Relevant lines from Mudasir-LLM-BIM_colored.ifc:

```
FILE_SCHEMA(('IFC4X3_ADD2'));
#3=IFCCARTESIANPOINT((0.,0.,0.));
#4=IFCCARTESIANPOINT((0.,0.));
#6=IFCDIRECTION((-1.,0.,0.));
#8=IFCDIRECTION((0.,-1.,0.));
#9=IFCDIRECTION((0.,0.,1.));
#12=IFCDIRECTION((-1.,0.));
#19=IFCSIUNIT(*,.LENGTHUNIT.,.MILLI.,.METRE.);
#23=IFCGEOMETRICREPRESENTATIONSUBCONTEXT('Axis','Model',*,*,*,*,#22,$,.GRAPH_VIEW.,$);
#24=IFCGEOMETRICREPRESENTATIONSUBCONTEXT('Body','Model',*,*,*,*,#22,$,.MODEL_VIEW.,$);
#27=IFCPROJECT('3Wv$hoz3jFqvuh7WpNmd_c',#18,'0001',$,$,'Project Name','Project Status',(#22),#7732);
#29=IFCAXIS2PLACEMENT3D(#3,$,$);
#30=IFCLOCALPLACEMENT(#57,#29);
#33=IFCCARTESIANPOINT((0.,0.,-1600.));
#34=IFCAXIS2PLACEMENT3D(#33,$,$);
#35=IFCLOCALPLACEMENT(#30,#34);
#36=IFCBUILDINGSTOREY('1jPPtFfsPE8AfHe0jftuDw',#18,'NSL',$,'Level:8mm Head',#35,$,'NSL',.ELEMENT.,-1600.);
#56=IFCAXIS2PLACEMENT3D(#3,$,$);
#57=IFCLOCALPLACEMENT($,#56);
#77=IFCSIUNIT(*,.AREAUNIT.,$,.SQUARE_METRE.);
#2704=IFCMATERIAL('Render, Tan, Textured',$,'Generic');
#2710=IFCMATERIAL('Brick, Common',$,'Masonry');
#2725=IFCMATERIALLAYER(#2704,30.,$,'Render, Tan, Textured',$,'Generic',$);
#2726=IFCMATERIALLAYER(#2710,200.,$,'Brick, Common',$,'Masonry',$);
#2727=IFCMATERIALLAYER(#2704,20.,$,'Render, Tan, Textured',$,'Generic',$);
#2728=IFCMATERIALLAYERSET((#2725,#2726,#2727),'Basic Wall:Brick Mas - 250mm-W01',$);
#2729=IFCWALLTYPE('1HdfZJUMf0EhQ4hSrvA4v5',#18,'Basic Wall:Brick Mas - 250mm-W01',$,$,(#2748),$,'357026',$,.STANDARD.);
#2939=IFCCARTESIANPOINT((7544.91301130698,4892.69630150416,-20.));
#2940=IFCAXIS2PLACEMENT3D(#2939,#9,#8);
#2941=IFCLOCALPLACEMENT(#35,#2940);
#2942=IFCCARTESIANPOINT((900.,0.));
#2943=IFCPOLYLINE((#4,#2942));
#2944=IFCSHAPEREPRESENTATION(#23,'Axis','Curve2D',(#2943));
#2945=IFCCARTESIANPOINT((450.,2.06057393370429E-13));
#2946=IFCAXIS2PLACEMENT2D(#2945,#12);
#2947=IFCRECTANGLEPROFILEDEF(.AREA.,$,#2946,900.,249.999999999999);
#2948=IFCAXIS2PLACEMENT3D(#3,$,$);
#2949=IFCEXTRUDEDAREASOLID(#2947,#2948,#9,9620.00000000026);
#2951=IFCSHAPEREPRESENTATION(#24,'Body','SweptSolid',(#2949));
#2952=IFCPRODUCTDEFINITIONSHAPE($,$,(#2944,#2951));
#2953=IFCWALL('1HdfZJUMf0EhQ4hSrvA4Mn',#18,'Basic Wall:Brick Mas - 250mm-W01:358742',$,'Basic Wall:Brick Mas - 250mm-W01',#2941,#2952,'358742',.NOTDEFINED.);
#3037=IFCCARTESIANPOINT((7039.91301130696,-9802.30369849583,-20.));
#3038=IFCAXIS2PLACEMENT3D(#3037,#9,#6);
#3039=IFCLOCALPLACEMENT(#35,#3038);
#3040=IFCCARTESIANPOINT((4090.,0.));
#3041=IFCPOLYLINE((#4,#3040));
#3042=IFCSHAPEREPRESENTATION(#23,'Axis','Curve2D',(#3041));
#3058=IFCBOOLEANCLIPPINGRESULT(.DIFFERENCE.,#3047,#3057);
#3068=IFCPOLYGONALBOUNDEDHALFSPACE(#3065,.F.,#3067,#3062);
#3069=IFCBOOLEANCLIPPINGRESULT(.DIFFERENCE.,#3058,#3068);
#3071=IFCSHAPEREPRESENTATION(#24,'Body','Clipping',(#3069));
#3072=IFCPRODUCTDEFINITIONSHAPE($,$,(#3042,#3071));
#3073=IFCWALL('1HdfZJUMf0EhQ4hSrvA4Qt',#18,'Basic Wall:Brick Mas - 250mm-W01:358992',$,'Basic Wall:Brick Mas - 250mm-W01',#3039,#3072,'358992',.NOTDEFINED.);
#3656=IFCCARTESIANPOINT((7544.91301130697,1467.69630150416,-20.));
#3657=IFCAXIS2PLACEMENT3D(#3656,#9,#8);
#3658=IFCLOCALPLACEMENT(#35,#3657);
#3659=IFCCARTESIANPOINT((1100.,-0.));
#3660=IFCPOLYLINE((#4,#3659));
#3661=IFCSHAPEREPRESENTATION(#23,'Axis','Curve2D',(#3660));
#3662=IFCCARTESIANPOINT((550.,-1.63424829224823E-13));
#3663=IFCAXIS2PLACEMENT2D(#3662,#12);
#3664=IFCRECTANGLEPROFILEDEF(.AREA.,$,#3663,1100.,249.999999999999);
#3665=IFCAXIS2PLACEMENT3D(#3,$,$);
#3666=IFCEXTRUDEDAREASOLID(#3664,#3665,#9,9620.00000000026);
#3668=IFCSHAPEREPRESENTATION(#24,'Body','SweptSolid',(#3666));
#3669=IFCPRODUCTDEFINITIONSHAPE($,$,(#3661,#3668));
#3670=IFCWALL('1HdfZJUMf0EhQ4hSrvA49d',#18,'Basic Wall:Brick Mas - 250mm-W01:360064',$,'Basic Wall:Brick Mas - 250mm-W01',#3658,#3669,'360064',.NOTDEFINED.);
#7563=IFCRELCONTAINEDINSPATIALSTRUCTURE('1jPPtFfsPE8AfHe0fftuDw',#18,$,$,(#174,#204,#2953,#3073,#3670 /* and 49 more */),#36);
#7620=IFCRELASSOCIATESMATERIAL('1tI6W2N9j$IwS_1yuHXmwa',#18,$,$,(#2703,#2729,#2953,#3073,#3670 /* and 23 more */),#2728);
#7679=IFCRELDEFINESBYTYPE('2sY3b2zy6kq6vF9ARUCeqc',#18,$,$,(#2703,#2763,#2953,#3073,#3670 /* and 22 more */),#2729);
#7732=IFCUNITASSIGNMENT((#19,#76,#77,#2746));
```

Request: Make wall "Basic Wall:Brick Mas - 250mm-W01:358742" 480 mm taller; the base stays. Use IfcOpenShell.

```python
import ifcopenshell
import ifcopenshell.geom
import ifcopenshell.util.representation
import ifcopenshell.util.shape
import ifcopenshell.util.unit

model = ifcopenshell.open("Mudasir-LLM-BIM_colored.ifc")
unit_scale = ifcopenshell.util.unit.calculate_unit_scale(model)
settings = ifcopenshell.geom.settings()


def volume(element):
    """Net volume in cubic metres, openings subtracted."""
    shape = ifcopenshell.geom.create_shape(settings, element)
    return ifcopenshell.util.shape.get_volume(shape.geometry)


wall = model.by_id(2953)
before = volume(wall)

body = ifcopenshell.util.representation.get_representation(wall, "Model", "Body")
solid = body.Items[0]
old_height = solid.Depth
solid.Depth += 0.48 / unit_scale
after = volume(wall)

print(f"height {old_height:g} -> {solid.Depth:g}, volume {before:.3f} -> {after:.3f} m3")

model.write("Mudasir-LLM-BIM_colored_rev.ifc")
```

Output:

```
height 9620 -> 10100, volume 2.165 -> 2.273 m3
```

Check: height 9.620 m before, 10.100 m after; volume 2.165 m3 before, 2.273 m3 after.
